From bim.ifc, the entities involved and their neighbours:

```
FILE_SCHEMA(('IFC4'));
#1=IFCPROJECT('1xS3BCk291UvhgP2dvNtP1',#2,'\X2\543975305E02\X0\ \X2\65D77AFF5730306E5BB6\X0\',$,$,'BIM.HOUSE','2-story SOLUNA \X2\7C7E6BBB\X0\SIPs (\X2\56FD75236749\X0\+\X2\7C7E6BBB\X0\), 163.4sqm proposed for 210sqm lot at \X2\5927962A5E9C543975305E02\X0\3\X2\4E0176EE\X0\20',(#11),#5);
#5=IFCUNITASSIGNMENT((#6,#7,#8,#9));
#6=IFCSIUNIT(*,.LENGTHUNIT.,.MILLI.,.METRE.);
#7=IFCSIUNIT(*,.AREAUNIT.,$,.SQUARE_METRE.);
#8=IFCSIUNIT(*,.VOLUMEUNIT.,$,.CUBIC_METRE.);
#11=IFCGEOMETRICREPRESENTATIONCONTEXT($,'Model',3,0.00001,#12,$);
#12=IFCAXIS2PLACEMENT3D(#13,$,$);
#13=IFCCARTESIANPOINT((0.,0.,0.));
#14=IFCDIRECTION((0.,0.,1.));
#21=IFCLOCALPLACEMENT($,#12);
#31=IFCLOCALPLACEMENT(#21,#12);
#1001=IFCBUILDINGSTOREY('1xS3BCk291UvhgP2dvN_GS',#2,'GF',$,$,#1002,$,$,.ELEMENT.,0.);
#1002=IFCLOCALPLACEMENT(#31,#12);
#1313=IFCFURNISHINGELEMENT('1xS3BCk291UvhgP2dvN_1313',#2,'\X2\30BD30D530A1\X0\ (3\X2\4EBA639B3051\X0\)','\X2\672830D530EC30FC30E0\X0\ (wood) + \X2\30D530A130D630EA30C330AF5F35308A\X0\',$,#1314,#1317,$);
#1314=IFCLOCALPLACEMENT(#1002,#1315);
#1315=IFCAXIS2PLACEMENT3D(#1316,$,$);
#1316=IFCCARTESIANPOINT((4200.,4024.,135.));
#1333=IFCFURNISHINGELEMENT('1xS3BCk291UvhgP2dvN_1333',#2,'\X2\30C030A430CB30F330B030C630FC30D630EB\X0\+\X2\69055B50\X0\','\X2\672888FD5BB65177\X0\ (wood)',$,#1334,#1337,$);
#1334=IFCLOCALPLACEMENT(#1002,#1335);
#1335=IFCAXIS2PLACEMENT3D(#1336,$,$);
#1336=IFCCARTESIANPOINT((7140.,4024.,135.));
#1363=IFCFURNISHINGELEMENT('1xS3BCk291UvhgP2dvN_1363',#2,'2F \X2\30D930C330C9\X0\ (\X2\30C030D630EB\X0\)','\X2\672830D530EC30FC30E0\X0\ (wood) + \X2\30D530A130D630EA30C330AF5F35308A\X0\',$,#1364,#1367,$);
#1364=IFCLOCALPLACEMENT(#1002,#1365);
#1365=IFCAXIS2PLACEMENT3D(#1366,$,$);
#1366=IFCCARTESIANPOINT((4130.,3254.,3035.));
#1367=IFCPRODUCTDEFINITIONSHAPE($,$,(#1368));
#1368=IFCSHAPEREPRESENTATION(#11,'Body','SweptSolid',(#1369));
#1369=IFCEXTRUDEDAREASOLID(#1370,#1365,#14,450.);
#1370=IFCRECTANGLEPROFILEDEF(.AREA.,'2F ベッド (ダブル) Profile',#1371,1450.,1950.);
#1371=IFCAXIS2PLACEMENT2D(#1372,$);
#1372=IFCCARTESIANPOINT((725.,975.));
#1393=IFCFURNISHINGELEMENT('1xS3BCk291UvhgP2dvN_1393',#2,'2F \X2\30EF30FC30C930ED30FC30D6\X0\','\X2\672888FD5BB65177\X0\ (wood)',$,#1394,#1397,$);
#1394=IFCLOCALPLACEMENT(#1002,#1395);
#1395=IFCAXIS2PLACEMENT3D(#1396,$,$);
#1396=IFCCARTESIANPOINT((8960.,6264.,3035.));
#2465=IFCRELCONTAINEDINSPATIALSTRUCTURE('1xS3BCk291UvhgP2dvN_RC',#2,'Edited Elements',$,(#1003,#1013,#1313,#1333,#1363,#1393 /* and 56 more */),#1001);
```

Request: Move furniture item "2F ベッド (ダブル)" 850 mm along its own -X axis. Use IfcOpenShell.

```python
import ifcopenshell
import ifcopenshell.api.geometry
import ifcopenshell.util.placement
import ifcopenshell.util.unit

model = ifcopenshell.open("bim.ifc")
unit_scale = ifcopenshell.util.unit.calculate_unit_scale(model)

item = model.by_id(1363)
matrix = ifcopenshell.util.placement.get_local_placement(item.ObjectPlacement)
matrix[:3, 3] -= matrix[:3, 0] * 0.85 / unit_scale
ifcopenshell.api.geometry.edit_object_placement(model, product=item, matrix=matrix, is_si=False)

print(ifcopenshell.util.placement.get_local_placement(item.ObjectPlacement).round(3) + 0.0)

model.write("bim_updated.ifc")
```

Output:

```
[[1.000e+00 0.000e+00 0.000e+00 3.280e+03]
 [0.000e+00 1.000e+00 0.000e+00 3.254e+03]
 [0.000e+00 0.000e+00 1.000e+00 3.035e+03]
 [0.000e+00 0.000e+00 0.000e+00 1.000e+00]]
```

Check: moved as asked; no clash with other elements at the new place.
